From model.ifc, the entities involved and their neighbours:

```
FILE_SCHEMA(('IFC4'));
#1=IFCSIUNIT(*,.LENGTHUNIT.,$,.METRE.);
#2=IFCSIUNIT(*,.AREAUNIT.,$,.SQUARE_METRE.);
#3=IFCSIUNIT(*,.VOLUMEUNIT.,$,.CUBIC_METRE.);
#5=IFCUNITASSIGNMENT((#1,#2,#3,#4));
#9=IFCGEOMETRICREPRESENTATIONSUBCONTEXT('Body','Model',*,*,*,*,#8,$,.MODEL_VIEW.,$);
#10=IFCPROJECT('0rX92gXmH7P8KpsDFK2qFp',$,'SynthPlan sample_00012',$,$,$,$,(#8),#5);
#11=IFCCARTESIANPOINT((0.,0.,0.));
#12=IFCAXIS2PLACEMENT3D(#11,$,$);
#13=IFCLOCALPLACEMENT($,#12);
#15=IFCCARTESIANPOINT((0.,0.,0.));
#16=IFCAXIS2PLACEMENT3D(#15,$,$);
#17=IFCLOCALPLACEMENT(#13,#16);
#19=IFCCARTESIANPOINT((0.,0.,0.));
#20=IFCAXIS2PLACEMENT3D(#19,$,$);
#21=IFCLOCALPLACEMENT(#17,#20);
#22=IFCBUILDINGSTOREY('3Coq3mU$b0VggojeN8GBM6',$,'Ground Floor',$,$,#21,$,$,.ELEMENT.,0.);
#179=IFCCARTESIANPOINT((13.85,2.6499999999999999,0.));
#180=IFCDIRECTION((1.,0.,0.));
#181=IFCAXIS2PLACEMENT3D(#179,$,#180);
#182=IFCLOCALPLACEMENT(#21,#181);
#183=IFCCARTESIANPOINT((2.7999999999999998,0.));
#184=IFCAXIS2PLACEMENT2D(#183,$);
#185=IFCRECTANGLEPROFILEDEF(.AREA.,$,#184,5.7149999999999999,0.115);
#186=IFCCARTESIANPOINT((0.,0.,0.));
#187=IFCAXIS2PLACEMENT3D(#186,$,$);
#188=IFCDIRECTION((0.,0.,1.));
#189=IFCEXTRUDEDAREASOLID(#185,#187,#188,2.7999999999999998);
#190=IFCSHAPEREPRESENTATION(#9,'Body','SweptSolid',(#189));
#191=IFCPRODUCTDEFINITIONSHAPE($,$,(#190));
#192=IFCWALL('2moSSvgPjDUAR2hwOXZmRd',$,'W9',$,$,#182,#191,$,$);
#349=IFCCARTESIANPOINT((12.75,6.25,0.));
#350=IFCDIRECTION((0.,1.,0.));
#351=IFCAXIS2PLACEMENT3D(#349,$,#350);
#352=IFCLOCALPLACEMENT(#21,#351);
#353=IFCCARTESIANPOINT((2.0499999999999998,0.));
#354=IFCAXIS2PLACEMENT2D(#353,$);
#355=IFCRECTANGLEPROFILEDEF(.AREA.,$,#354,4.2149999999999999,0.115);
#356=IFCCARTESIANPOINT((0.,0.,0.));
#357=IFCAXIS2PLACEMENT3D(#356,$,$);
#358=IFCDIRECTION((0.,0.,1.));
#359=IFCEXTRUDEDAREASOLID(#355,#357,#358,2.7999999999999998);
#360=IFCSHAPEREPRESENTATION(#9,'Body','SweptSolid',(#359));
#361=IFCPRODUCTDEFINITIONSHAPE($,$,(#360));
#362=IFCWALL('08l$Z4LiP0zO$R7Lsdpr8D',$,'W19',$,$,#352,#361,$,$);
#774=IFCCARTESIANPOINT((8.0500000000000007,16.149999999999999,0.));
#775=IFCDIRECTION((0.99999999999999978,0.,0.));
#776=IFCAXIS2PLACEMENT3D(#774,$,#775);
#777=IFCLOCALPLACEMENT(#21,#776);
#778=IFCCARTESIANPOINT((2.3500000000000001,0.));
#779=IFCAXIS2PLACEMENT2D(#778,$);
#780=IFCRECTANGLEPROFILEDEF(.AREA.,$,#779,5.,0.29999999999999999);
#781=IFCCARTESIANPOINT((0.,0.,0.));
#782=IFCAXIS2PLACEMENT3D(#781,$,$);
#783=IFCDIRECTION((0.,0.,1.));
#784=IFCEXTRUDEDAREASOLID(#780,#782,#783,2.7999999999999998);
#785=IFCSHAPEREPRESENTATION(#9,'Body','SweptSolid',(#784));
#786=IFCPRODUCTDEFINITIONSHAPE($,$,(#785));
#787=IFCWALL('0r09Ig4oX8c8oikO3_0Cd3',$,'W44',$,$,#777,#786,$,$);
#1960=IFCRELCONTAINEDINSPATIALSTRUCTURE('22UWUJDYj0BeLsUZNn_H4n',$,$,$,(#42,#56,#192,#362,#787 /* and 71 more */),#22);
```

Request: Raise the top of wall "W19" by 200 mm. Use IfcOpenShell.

```python
import ifcopenshell
import ifcopenshell.geom
import ifcopenshell.util.representation
import ifcopenshell.util.shape
import ifcopenshell.util.unit

model = ifcopenshell.open("model.ifc")
unit_scale = ifcopenshell.util.unit.calculate_unit_scale(model)
settings = ifcopenshell.geom.settings()


def volume(element):
    """Net volume in cubic metres, openings subtracted."""
    shape = ifcopenshell.geom.create_shape(settings, element)
    return ifcopenshell.util.shape.get_volume(shape.geometry)


wall = model.by_guid("08l$Z4LiP0zO$R7Lsdpr8D")
before = volume(wall)

body = ifcopenshell.util.representation.get_representation(wall, "Model", "Body")
solid = body.Items[0]
old_height = solid.Depth
solid.Depth += 0.2 / unit_scale
after = volume(wall)

print(f"height {old_height:g} -> {solid.Depth:g}, volume {before:.3f} -> {after:.3f} m3")

model.write("model_rev.ifc")
```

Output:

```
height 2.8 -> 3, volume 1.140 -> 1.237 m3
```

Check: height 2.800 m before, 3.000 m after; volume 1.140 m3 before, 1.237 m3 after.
